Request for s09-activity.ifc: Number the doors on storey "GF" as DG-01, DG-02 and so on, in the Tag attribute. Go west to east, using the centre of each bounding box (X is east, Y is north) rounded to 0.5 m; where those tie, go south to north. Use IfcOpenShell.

First a look at what the model holds.

```python
import ifcopenshell
import ifcopenshell.util.element
import ifcopenshell.util.placement

model = ifcopenshell.open("s09-activity.ifc")
print(model.schema)
storey = next(s for s in model.by_type("IfcBuildingStorey") if s.Name == "GF")
doors = [e for e in ifcopenshell.util.element.get_decomposition(storey) if e.is_a("IfcDoor")]
for e in sorted(doors, key=lambda e: e.id()):
    origin = ifcopenshell.util.placement.get_local_placement(e.ObjectPlacement)[:3, 3]
    print(e.id(), e.Tag, e.Name, origin.round(2) + 0.0, sep=" | ")
```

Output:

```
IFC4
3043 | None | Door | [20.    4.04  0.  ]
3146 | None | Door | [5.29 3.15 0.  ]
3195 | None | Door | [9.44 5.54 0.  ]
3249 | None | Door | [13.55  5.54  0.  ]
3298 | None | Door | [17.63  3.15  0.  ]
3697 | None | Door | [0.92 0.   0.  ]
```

```python
import ifcopenshell
import ifcopenshell.geom
import ifcopenshell.util.element
import ifcopenshell.util.shape

model = ifcopenshell.open("s09-activity.ifc")
settings = ifcopenshell.geom.settings()
settings.set("use-world-coords", True)


def centre(element):
    shape = ifcopenshell.geom.create_shape(settings, element)
    return ifcopenshell.util.shape.get_bbox_centroid(shape.geometry)


storey = next(s for s in model.by_type("IfcBuildingStorey") if s.Name == "GF")
doors = [e for e in ifcopenshell.util.element.get_decomposition(storey) if e.is_a("IfcDoor")]

# Insertion points can sit at a corner or the storey origin, so sort by the geometry (in metres).
centres = {e: centre(e) for e in doors}
doors.sort(key=lambda e: (round(centres[e][0] / 0.5), centres[e][1]))

for i, e in enumerate(doors, start=1):
    number = f"DG-{i:02d}"
    e.Tag = number
    print(e.id(), number)

model.write("s09-activity_edited.ifc")
```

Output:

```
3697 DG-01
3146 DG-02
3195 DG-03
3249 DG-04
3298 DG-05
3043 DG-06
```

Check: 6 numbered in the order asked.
